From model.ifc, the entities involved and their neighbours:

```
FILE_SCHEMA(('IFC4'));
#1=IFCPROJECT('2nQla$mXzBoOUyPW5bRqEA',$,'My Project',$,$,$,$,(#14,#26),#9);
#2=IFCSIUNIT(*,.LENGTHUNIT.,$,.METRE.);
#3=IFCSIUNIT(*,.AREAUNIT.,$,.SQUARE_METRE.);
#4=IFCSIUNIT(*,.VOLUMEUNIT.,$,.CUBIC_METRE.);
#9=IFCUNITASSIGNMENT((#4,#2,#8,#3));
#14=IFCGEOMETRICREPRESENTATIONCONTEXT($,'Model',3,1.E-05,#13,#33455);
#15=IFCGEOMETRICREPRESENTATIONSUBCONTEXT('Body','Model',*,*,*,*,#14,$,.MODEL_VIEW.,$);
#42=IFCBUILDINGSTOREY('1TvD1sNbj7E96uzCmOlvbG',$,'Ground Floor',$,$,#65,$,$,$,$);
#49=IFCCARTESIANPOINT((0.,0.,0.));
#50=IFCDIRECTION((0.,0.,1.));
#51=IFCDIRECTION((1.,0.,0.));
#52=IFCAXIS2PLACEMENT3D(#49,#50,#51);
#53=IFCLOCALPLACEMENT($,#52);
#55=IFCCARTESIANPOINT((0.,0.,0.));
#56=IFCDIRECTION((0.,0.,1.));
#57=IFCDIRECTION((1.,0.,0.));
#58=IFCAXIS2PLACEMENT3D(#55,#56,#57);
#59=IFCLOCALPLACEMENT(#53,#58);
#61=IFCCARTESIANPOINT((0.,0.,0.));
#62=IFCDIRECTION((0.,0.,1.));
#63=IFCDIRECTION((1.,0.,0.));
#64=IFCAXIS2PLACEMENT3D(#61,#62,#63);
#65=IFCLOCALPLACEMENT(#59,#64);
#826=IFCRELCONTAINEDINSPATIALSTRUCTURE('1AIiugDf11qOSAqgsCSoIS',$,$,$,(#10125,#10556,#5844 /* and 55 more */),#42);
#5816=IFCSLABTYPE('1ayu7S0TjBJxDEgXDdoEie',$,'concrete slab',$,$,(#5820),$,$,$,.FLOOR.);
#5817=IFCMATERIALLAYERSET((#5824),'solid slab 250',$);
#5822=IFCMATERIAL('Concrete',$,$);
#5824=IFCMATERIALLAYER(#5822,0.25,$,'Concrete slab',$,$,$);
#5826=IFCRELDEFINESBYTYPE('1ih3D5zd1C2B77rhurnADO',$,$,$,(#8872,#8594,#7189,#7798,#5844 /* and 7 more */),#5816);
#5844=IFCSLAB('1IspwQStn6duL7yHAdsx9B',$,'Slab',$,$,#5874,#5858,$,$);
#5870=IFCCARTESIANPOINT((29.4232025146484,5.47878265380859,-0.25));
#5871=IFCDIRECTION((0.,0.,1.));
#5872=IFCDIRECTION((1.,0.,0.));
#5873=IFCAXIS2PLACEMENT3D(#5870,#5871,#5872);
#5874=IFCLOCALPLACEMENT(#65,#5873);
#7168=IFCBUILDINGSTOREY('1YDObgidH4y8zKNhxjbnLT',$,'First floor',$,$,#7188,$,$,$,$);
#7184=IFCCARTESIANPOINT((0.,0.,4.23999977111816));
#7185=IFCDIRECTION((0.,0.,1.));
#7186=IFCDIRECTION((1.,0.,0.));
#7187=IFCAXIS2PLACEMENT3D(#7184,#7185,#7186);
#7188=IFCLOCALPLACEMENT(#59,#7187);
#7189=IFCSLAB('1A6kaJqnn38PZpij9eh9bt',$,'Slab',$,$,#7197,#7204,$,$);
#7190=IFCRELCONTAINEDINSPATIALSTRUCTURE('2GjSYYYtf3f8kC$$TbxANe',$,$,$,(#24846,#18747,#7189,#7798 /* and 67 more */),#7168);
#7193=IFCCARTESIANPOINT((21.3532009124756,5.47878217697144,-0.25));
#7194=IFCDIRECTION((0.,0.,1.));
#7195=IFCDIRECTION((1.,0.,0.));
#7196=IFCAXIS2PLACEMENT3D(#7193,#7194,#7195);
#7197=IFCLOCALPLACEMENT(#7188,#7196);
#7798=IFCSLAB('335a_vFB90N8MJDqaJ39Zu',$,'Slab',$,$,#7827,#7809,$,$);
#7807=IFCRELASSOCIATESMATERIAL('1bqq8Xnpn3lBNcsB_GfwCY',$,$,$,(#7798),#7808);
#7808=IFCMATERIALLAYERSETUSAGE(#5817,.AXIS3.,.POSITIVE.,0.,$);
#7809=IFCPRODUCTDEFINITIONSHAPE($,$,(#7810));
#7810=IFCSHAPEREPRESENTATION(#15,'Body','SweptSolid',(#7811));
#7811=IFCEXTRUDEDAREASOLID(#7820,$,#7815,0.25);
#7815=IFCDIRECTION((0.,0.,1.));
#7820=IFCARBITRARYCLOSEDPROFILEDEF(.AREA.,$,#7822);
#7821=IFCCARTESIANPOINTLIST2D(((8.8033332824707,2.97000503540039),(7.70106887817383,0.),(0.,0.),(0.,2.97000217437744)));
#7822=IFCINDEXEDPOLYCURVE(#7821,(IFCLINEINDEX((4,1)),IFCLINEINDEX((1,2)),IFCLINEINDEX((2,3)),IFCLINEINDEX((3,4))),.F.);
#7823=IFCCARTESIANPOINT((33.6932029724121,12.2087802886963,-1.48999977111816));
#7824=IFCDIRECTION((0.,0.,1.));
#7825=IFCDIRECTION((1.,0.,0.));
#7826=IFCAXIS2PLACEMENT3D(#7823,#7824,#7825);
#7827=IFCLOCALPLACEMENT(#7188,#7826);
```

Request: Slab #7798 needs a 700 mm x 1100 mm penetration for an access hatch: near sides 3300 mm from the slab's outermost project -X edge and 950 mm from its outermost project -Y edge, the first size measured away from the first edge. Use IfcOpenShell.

```python
import numpy as np
import ifcopenshell
import ifcopenshell.api.feature
import ifcopenshell.api.geometry
import ifcopenshell.api.root
import ifcopenshell.geom
import ifcopenshell.util.placement
import ifcopenshell.util.representation
import ifcopenshell.util.shape
import ifcopenshell.util.unit

model = ifcopenshell.open("model.ifc")
unit_scale = ifcopenshell.util.unit.calculate_unit_scale(model)
settings = ifcopenshell.geom.settings()


def volume(element):
    """Net volume in cubic metres, openings subtracted."""
    shape = ifcopenshell.geom.create_shape(settings, element)
    return ifcopenshell.util.shape.get_volume(shape.geometry)


slab = model.by_guid("335a_vFB90N8MJDqaJ39Zu")
before = volume(slab)

# Extent in the slab's own axes, in metres. The edges named are its -X and -Y sides.
slab_shape = ifcopenshell.geom.create_shape(settings, slab)
vertices = ifcopenshell.util.shape.get_vertices(slab_shape.geometry)
x_min, y_min, bottom = vertices.min(axis=0)
top = vertices[:, 2].max()

opening = ifcopenshell.api.root.create_entity(model, ifc_class="IfcOpeningElement", name="Access hatch opening", predefined_type="OPENING")
context = ifcopenshell.util.representation.get_context(model, "Model", "Body", "MODEL_VIEW")
width, depth = 0.7, 1.1
outline = [(0.0, 0.0), (width, 0.0), (width, depth), (0.0, depth), (0.0, 0.0)]
# Overshoot both faces by 50 mm so the cut is clean.
shape = ifcopenshell.api.geometry.add_slab_representation(
    model, context=context, depth=top - bottom + 0.1, polyline=outline
)
ifcopenshell.api.geometry.assign_representation(model, product=opening, representation=shape)

matrix = ifcopenshell.util.placement.get_local_placement(slab.ObjectPlacement)
matrix[:, 3] = matrix @ np.append(np.array([x_min + 3.3, y_min + 0.95, bottom - 0.05]) / unit_scale, 1.0)
ifcopenshell.api.geometry.edit_object_placement(model, product=opening, matrix=matrix, is_si=False)
ifcopenshell.api.feature.add_feature(model, feature=opening, element=slab)

after = volume(slab)

print(f"slab volume {before:.3f} -> {after:.3f} m3")

model.write("model_v2.ifc")
```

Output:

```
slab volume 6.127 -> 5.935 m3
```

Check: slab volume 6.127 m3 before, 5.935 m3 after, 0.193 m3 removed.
